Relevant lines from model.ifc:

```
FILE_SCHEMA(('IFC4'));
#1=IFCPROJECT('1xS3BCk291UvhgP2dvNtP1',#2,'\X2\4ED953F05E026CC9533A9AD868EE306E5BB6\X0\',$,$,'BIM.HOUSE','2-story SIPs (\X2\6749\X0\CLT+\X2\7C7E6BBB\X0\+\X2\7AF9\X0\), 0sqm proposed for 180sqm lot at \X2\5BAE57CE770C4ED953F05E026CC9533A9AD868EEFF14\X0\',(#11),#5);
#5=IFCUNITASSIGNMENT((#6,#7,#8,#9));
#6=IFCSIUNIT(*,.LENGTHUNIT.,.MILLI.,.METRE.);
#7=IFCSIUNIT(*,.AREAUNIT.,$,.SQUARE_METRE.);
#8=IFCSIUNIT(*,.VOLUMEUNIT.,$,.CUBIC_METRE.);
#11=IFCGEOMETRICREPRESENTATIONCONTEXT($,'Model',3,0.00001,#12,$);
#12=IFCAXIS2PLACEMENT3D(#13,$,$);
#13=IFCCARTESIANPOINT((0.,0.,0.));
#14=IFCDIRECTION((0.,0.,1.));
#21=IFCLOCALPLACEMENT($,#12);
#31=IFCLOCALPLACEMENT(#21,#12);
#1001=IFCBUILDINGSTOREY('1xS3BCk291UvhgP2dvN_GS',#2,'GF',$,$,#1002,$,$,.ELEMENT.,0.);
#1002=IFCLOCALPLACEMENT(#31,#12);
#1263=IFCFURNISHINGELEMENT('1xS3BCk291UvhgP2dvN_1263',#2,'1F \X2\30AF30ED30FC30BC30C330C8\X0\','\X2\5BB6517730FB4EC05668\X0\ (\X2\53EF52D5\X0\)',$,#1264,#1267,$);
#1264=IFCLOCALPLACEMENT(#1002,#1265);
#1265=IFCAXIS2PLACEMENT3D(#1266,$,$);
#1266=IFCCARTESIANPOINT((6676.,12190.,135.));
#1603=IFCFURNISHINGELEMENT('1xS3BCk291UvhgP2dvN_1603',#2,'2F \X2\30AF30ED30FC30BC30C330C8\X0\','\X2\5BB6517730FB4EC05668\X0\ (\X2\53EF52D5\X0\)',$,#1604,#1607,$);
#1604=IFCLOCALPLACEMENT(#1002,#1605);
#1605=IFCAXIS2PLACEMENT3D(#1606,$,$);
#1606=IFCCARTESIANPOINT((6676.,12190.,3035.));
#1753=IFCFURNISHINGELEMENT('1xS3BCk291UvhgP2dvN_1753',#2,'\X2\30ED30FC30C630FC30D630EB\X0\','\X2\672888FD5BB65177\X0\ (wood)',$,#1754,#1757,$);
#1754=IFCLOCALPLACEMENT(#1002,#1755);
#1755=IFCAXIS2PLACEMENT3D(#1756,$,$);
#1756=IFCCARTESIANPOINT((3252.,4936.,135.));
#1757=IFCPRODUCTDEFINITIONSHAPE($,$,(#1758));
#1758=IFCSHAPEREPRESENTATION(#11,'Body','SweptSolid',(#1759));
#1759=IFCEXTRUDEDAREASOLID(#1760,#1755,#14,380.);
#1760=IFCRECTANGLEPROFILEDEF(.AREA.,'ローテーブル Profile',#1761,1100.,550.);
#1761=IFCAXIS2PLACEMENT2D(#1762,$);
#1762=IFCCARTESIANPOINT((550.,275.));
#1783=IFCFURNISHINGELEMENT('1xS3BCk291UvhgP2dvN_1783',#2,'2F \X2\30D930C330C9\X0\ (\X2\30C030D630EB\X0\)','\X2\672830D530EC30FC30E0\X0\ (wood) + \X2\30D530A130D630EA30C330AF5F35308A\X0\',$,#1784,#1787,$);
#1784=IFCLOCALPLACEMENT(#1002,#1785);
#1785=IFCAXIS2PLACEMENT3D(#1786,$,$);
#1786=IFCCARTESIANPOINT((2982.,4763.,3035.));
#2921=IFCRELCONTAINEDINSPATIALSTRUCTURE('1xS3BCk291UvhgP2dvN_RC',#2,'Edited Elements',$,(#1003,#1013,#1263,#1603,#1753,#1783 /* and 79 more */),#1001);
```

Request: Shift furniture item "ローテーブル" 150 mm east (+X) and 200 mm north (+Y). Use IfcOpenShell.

```python
import ifcopenshell
import ifcopenshell.api.geometry
import ifcopenshell.util.placement
import ifcopenshell.util.unit

model = ifcopenshell.open("model.ifc")
unit_scale = ifcopenshell.util.unit.calculate_unit_scale(model)

item = model.by_guid("1xS3BCk291UvhgP2dvN_1753")
matrix = ifcopenshell.util.placement.get_local_placement(item.ObjectPlacement)
matrix[0, 3] += 0.15 / unit_scale
matrix[1, 3] += 0.2 / unit_scale
ifcopenshell.api.geometry.edit_object_placement(model, product=item, matrix=matrix, is_si=False)

print(ifcopenshell.util.placement.get_local_placement(item.ObjectPlacement).round(3) + 0.0)

model.write("model_v2.ifc")
```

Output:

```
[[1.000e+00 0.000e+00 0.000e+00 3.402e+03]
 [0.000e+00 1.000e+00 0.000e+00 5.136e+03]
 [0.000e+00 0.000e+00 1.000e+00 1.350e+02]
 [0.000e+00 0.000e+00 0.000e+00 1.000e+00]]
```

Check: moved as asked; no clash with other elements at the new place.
